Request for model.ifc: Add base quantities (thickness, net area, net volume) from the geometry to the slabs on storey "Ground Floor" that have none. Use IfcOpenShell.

First a look at what the model holds.

```python
import ifcopenshell
import ifcopenshell.util.element
import ifcopenshell.util.unit

model = ifcopenshell.open("model.ifc")
print(model.schema)
for unit_type in ("LENGTHUNIT", "AREAUNIT", "VOLUMEUNIT"):
    print(unit_type, ifcopenshell.util.unit.calculate_unit_scale(model, unit_type))
storey = next(s for s in model.by_type("IfcBuildingStorey") if s.Name == "Ground Floor")
slabs = [e for e in ifcopenshell.util.element.get_decomposition(storey) if e.is_a("IfcSlab")]
for e in sorted(slabs, key=lambda e: e.id()):
    print(e.id(), e.is_a(), e.Name, list(ifcopenshell.util.element.get_psets(e, qtos_only=True)), sep=" | ")
```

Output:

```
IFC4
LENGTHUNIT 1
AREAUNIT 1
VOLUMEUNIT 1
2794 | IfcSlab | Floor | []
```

```python
import ifcopenshell
import ifcopenshell.api.pset
import ifcopenshell.geom
import ifcopenshell.util.element
import ifcopenshell.util.shape
import ifcopenshell.util.unit

model = ifcopenshell.open("model.ifc")
unit_scale = ifcopenshell.util.unit.calculate_unit_scale(model)
area_scale = ifcopenshell.util.unit.calculate_unit_scale(model, "AREAUNIT")
volume_scale = ifcopenshell.util.unit.calculate_unit_scale(model, "VOLUMEUNIT")
settings = ifcopenshell.geom.settings()

storey = next(s for s in model.by_type("IfcBuildingStorey") if s.Name == "Ground Floor")
slabs = [e for e in ifcopenshell.util.element.get_decomposition(storey) if e.is_a("IfcSlab")]

for e in sorted(slabs, key=lambda e: e.id()):
    if ifcopenshell.util.element.get_psets(e, qtos_only=True, should_inherit=False):
        continue
    # Geometry comes back in metres, in the element's own axes.
    shape = ifcopenshell.geom.create_shape(settings, e)
    values = {
        "Width": ifcopenshell.util.shape.get_z(shape.geometry) / unit_scale,
        "NetArea": ifcopenshell.util.shape.get_footprint_area(shape.geometry) / area_scale,
        "NetVolume": ifcopenshell.util.shape.get_volume(shape.geometry) / volume_scale,
    }
    qto = ifcopenshell.api.pset.add_qto(model, product=e, name="Qto_SlabBaseQuantities")
    ifcopenshell.api.pset.edit_qto(model, qto=qto, properties=values)
    print(e.id(), {k: round(v, 3) for k, v in values.items()})

model.write("model_rev.ifc")
```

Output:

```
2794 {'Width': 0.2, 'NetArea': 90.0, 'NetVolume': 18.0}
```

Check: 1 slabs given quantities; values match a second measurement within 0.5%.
